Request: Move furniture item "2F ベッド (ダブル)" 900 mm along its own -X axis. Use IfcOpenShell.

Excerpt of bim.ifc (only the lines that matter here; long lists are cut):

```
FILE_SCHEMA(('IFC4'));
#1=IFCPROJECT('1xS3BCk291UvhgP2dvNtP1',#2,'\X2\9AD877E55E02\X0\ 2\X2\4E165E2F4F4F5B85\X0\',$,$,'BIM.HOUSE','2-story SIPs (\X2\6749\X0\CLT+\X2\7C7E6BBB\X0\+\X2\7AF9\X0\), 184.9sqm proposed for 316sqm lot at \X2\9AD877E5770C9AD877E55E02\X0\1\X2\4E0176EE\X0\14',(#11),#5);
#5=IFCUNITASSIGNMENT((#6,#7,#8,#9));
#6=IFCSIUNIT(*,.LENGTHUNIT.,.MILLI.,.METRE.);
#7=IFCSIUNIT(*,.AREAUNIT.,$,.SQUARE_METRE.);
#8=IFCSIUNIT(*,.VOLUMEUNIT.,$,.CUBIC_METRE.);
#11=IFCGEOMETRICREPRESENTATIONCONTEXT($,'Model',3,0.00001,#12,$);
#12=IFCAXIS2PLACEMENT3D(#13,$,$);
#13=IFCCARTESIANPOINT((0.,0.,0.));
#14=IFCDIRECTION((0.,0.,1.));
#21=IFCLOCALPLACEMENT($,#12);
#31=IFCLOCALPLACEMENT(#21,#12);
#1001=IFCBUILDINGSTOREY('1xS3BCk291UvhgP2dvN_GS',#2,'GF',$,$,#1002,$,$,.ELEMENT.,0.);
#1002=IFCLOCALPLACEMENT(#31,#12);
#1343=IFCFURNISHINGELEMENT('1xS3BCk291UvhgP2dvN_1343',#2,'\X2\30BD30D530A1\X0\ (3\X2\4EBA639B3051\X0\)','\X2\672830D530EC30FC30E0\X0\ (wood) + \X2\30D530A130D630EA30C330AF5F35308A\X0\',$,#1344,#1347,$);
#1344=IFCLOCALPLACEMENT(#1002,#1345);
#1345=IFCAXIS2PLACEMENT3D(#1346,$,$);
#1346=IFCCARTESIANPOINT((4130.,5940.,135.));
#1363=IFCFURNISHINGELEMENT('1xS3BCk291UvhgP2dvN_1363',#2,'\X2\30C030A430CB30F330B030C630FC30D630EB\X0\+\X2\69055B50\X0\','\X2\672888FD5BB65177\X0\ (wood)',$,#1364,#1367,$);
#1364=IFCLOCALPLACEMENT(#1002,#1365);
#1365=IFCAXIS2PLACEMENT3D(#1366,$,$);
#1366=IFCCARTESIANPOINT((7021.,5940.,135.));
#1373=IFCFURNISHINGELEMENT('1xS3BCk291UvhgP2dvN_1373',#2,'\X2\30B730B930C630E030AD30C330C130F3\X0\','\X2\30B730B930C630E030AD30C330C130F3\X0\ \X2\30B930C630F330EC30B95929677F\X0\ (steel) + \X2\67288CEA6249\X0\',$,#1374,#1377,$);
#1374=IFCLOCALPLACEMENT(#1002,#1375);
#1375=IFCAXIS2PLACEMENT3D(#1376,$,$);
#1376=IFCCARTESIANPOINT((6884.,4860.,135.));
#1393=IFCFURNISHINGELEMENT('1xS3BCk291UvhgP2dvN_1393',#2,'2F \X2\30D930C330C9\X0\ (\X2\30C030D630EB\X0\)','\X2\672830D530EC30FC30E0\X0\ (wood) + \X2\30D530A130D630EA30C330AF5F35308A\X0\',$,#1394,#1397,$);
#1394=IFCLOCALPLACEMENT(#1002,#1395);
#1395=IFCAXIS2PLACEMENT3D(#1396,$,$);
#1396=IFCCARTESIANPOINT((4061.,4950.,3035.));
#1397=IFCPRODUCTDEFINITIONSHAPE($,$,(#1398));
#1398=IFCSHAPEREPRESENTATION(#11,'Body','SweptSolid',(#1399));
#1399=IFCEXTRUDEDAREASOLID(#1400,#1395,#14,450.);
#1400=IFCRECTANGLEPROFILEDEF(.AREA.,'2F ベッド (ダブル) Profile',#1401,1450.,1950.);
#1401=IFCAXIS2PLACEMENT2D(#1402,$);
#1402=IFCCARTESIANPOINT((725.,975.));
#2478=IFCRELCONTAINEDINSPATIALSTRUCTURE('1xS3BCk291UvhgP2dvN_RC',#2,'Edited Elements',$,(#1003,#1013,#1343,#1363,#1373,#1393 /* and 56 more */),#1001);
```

```python
import ifcopenshell
import ifcopenshell.api.geometry
import ifcopenshell.util.placement

model = ifcopenshell.open("bim.ifc")

item = model.by_guid("1xS3BCk291UvhgP2dvN_1393")
matrix = ifcopenshell.util.placement.get_local_placement(item.ObjectPlacement)
matrix[:3, 3] -= matrix[:3, 0] * 900.0
ifcopenshell.api.geometry.edit_object_placement(model, product=item, matrix=matrix, is_si=False)

print(ifcopenshell.util.placement.get_local_placement(item.ObjectPlacement).round(3) + 0.0)

model.write("bim_edited.ifc")
```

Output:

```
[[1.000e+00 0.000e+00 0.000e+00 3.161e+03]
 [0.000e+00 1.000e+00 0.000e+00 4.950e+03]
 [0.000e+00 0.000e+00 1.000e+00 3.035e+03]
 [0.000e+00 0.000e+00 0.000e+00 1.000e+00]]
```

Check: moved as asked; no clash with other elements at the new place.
